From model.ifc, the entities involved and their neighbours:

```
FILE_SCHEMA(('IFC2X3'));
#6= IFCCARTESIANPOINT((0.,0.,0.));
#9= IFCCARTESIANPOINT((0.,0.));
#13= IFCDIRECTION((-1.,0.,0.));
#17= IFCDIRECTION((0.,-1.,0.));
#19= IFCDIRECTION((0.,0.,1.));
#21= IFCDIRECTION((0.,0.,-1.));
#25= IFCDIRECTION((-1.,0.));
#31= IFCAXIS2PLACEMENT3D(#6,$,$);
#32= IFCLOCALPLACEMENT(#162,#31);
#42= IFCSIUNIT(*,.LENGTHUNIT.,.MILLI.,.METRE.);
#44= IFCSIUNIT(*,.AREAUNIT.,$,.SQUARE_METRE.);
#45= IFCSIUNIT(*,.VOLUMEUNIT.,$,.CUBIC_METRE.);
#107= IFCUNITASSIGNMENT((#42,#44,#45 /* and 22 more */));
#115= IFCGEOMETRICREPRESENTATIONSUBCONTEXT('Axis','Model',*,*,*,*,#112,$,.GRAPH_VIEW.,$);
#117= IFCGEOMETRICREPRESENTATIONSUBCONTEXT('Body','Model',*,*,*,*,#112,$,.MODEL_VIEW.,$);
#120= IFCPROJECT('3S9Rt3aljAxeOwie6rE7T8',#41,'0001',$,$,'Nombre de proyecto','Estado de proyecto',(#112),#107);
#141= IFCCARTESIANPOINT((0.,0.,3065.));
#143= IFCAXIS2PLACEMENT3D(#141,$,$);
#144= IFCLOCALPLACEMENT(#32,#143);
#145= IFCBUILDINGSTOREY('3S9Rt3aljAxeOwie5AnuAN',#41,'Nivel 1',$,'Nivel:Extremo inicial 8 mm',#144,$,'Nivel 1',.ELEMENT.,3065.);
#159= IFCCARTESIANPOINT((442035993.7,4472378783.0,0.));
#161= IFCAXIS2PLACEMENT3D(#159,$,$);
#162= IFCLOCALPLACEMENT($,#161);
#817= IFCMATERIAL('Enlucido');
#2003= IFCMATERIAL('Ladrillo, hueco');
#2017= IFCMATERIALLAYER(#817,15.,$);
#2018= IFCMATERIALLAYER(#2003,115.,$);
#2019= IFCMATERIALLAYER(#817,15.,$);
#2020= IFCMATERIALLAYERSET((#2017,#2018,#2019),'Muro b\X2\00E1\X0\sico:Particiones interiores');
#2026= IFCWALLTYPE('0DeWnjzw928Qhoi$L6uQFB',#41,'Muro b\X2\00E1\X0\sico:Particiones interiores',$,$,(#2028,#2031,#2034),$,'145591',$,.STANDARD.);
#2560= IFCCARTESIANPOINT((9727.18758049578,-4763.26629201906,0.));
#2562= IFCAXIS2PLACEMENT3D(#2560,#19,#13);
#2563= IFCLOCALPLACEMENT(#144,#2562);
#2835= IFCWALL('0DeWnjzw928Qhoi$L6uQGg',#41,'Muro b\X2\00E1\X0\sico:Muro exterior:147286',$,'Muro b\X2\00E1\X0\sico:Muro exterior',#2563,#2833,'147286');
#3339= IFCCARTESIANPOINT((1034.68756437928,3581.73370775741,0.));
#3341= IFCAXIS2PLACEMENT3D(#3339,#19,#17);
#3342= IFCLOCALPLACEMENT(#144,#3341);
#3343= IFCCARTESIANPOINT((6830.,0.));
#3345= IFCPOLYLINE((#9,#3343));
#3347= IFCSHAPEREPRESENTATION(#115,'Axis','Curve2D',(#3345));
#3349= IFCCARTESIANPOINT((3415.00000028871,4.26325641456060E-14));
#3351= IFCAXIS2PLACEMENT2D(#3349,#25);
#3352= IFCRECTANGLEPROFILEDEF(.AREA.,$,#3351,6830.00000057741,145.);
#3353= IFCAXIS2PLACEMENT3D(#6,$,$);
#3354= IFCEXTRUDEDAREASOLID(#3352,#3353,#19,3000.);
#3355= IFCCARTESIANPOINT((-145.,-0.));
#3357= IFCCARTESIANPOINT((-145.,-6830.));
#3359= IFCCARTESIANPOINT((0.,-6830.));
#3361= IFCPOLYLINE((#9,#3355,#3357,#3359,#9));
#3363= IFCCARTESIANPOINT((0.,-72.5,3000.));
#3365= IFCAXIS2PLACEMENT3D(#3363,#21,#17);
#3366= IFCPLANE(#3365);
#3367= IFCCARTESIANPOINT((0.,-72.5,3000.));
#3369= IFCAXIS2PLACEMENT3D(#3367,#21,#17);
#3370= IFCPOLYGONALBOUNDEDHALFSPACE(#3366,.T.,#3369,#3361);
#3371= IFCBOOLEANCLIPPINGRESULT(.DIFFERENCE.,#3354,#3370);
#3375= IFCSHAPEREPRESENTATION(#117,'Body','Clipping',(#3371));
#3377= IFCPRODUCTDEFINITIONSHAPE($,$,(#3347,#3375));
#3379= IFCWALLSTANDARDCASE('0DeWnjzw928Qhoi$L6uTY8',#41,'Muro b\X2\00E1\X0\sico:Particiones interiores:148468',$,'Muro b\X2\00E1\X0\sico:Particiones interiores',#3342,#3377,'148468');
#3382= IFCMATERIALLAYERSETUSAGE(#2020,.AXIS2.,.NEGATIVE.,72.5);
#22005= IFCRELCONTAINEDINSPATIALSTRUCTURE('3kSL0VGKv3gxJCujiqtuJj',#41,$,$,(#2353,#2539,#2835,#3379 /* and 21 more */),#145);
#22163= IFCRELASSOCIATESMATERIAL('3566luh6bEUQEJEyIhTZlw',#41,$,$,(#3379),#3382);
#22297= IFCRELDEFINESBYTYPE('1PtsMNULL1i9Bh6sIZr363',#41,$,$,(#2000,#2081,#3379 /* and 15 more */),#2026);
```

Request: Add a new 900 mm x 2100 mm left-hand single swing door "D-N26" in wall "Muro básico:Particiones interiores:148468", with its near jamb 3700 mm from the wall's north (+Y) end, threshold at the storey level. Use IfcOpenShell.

```python
import numpy as np
import ifcopenshell
import ifcopenshell.api.feature
import ifcopenshell.api.geometry
import ifcopenshell.api.root
import ifcopenshell.api.spatial
import ifcopenshell.api.type
import ifcopenshell.geom
import ifcopenshell.util.element
import ifcopenshell.util.placement
import ifcopenshell.util.representation
import ifcopenshell.util.shape
import ifcopenshell.util.unit

model = ifcopenshell.open("model.ifc")
unit_scale = ifcopenshell.util.unit.calculate_unit_scale(model)
settings = ifcopenshell.geom.settings()


def volume(element):
    """Net volume in cubic metres, openings subtracted."""
    shape = ifcopenshell.geom.create_shape(settings, element)
    return ifcopenshell.util.shape.get_volume(shape.geometry)


wall = model.by_guid("0DeWnjzw928Qhoi$L6uTY8")
storey = ifcopenshell.util.element.get_container(wall, ifc_class="IfcBuildingStorey")
context = ifcopenshell.util.representation.get_context(model, "Model", "Body", "MODEL_VIEW")
before = volume(wall)

width, height, from_end, sill = 0.9, 2.1, 3.7, 0.0  # metres

# The wall runs along its own X axis, and the end named is its -X end.
wall_shape = ifcopenshell.geom.create_shape(settings, wall)
x, y, z = ifcopenshell.util.shape.get_vertices(wall_shape.geometry).T
start = x.min() + from_end
face, thickness = float(y.min()), float(y.max() - y.min())
wall_matrix = ifcopenshell.util.placement.get_local_placement(wall.ObjectPlacement)
level = ifcopenshell.util.placement.get_local_placement(storey.ObjectPlacement)[2, 3]


def in_wall(x, y):
    """Placement at x, y metres in the wall's axes, at sill height."""
    matrix = wall_matrix.copy()
    matrix[:, 3] = wall_matrix @ np.array([x / unit_scale, y / unit_scale, 0.0, 1.0])
    matrix[2, 3] = level + sill / unit_scale
    return matrix


# Opening: a box that overshoots both wall faces by 50 mm.
opening = ifcopenshell.api.root.create_entity(model, ifc_class="IfcOpeningElement")
box = ifcopenshell.api.geometry.add_wall_representation(
    model, context=context, length=width, height=height, thickness=thickness + 0.1
)
ifcopenshell.api.geometry.assign_representation(model, product=opening, representation=box)
ifcopenshell.api.geometry.edit_object_placement(model, product=opening, matrix=in_wall(start, face - 0.05), is_si=False)
ifcopenshell.api.feature.add_feature(model, feature=opening, element=wall)

door = ifcopenshell.api.root.create_entity(model, ifc_class="IfcDoor", name="D-N26")
door.OverallWidth, door.OverallHeight = width / unit_scale, height / unit_scale
body = ifcopenshell.api.geometry.add_door_representation(
    model,
    context=context,
    overall_width=door.OverallWidth,
    overall_height=door.OverallHeight,
    operation_type="SINGLE_SWING_LEFT",
    lining_properties={"LiningDepth": thickness / unit_scale, "ThresholdDepth": thickness / unit_scale},
)
ifcopenshell.api.geometry.assign_representation(model, product=door, representation=body)
ifcopenshell.api.spatial.assign_container(model, products=[door], relating_structure=storey)
fills = ifcopenshell.api.feature.add_filling(model, opening=opening, element=door)
fills.OwnerHistory = door.OwnerHistory  # required in IFC2X3

# IFC2X3 keeps the operation on the door style.
style = ifcopenshell.api.root.create_entity(model, ifc_class="IfcDoorStyle", name="D-N26")
style.OperationType, style.ConstructionType = "SINGLE_SWING_LEFT", "NOTDEFINED"
style.ParameterTakesPrecedence = style.Sizeable = False
ifcopenshell.api.type.assign_type(model, related_objects=[door], relating_type=style)

# The lining spans the wall, so the door starts at the wall face.
ifcopenshell.api.geometry.edit_object_placement(model, product=door, matrix=in_wall(start, face), is_si=False)

after = volume(wall)

print(f"wall volume {before:.3f} -> {after:.3f} m3")

model.write("model_edited.ifc")
```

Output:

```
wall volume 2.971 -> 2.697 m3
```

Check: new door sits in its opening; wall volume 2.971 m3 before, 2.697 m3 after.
